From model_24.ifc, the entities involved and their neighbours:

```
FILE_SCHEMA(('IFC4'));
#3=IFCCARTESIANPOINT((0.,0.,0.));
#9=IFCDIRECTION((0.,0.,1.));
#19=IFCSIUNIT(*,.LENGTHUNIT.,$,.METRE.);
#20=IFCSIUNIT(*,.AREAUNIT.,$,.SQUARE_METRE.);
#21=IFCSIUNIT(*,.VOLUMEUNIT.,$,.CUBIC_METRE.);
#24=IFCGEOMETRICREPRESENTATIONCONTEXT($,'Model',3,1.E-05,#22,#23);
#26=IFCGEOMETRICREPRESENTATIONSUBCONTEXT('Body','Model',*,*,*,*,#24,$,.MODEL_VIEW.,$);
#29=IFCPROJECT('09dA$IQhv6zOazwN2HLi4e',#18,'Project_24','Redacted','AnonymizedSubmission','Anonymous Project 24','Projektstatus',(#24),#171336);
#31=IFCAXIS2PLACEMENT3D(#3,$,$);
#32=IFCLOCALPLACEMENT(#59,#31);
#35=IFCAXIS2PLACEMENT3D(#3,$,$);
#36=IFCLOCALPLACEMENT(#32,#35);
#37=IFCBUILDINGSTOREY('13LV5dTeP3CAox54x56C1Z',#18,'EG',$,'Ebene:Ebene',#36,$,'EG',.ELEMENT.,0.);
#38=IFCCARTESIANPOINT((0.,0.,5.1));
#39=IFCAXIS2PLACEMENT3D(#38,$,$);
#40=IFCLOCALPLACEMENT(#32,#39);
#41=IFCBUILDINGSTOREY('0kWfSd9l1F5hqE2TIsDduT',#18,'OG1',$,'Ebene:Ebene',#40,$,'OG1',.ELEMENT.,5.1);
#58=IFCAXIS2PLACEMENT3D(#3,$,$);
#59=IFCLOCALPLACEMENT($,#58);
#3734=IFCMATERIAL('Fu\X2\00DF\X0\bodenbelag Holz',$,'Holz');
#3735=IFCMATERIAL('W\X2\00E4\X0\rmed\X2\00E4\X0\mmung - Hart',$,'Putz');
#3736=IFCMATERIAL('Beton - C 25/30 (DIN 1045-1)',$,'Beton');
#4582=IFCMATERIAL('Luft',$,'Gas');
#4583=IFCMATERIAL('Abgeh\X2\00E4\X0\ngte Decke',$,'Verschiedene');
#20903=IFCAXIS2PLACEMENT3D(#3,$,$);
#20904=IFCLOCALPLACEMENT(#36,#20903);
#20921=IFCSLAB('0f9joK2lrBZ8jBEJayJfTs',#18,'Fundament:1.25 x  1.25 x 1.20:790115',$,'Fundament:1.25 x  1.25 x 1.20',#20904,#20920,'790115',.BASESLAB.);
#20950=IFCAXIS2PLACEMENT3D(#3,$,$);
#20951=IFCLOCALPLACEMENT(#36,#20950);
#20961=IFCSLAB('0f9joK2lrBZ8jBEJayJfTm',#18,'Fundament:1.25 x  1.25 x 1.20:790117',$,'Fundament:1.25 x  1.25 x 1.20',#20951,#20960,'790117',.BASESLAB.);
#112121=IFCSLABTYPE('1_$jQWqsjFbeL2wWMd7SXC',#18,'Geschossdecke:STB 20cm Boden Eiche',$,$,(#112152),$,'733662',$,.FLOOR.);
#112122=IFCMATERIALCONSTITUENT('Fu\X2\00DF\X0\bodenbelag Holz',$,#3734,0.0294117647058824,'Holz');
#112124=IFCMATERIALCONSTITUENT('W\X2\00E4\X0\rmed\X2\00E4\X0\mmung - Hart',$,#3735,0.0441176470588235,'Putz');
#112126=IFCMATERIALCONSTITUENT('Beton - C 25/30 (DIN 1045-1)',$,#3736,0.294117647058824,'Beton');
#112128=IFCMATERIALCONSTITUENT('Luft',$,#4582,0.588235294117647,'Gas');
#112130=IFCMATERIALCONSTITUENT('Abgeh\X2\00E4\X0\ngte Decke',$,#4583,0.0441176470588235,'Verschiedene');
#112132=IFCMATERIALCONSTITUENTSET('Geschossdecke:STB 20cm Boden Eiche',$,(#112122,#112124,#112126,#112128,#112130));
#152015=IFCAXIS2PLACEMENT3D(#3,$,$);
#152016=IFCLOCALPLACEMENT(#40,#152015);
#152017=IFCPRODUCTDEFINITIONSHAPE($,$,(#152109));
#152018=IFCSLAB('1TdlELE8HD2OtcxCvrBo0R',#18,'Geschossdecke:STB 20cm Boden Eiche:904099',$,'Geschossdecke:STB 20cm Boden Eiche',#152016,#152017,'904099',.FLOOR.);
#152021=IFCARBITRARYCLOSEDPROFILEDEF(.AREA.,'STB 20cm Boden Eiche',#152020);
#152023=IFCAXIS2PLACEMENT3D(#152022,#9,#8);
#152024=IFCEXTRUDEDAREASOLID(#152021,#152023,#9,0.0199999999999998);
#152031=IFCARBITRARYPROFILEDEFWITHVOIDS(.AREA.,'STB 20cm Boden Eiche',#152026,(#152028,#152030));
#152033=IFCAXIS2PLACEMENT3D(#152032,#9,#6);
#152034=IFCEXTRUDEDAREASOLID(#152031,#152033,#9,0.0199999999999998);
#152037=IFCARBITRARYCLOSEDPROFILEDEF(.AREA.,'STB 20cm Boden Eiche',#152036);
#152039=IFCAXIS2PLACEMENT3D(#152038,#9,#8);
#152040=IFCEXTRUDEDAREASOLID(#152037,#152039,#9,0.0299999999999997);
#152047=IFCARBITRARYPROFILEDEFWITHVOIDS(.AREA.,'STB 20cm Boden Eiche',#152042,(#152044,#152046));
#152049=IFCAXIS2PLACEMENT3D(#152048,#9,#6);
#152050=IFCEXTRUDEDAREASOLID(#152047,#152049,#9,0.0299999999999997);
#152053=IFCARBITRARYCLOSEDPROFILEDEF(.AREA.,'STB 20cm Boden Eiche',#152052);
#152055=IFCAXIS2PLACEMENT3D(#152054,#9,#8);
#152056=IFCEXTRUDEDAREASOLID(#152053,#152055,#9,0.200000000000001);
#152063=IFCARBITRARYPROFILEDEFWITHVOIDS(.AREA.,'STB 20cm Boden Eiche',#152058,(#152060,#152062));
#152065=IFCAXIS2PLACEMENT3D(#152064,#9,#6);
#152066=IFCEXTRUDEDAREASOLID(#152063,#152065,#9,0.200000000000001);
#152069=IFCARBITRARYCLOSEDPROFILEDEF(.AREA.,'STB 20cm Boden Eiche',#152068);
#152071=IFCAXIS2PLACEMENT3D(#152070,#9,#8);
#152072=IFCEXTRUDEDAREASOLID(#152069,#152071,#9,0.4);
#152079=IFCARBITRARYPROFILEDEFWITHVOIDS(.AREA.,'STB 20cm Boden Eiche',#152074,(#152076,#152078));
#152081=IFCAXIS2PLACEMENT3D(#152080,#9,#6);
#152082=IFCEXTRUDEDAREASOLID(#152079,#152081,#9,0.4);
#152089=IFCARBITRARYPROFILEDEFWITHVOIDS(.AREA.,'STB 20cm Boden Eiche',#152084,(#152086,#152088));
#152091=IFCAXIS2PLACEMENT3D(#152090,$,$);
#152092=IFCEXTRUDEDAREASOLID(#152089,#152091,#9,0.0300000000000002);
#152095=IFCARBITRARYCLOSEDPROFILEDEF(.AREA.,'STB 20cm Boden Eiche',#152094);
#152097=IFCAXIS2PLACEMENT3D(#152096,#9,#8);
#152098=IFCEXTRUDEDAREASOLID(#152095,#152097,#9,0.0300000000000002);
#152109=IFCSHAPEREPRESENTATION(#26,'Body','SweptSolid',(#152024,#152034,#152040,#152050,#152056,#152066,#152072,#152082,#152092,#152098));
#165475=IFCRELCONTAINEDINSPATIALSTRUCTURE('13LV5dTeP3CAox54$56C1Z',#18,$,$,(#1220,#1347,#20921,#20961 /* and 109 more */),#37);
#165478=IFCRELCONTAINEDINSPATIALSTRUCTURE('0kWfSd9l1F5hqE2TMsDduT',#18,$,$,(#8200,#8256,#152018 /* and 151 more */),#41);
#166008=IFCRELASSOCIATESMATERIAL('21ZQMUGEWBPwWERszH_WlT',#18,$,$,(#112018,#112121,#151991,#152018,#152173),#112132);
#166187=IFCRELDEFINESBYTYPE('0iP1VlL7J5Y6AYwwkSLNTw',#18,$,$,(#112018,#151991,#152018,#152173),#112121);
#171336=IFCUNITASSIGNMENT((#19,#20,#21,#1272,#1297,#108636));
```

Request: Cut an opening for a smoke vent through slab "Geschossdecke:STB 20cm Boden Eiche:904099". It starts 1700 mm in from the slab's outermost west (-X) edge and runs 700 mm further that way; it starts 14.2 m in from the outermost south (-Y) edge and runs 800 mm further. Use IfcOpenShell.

```python
import numpy as np
import ifcopenshell
import ifcopenshell.api.feature
import ifcopenshell.api.geometry
import ifcopenshell.api.root
import ifcopenshell.geom
import ifcopenshell.util.placement
import ifcopenshell.util.representation
import ifcopenshell.util.shape
import ifcopenshell.util.unit

model = ifcopenshell.open("model_24.ifc")
unit_scale = ifcopenshell.util.unit.calculate_unit_scale(model)
settings = ifcopenshell.geom.settings()


def volume(element):
    """Net volume in cubic metres, openings subtracted."""
    shape = ifcopenshell.geom.create_shape(settings, element)
    return ifcopenshell.util.shape.get_volume(shape.geometry)


slab = model.by_id(152018)
before = volume(slab)

# Extent in the slab's own axes, in metres. The edges named are its -X and -Y sides.
slab_shape = ifcopenshell.geom.create_shape(settings, slab)
vertices = ifcopenshell.util.shape.get_vertices(slab_shape.geometry)
x_min, y_min, bottom = vertices.min(axis=0)
top = vertices[:, 2].max()

opening = ifcopenshell.api.root.create_entity(model, ifc_class="IfcOpeningElement", name="Smoke vent opening", predefined_type="OPENING")
context = ifcopenshell.util.representation.get_context(model, "Model", "Body", "MODEL_VIEW")
width, depth = 0.7, 0.8
outline = [(0.0, 0.0), (width, 0.0), (width, depth), (0.0, depth), (0.0, 0.0)]
# Overshoot both faces by 50 mm so the cut is clean.
shape = ifcopenshell.api.geometry.add_slab_representation(
    model, context=context, depth=top - bottom + 0.1, polyline=outline
)
ifcopenshell.api.geometry.assign_representation(model, product=opening, representation=shape)

matrix = ifcopenshell.util.placement.get_local_placement(slab.ObjectPlacement)
matrix[:, 3] = matrix @ np.append(np.array([x_min + 1.7, y_min + 14.2, bottom - 0.05]) / unit_scale, 1.0)
ifcopenshell.api.geometry.edit_object_placement(model, product=opening, matrix=matrix, is_si=False)
ifcopenshell.api.feature.add_feature(model, feature=opening, element=slab)

after = volume(slab)

print(f"slab volume {before:.3f} -> {after:.3f} m3")

model.write("model_24_v2.ifc")
```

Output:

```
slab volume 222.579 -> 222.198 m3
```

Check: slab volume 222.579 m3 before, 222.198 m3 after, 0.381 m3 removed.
